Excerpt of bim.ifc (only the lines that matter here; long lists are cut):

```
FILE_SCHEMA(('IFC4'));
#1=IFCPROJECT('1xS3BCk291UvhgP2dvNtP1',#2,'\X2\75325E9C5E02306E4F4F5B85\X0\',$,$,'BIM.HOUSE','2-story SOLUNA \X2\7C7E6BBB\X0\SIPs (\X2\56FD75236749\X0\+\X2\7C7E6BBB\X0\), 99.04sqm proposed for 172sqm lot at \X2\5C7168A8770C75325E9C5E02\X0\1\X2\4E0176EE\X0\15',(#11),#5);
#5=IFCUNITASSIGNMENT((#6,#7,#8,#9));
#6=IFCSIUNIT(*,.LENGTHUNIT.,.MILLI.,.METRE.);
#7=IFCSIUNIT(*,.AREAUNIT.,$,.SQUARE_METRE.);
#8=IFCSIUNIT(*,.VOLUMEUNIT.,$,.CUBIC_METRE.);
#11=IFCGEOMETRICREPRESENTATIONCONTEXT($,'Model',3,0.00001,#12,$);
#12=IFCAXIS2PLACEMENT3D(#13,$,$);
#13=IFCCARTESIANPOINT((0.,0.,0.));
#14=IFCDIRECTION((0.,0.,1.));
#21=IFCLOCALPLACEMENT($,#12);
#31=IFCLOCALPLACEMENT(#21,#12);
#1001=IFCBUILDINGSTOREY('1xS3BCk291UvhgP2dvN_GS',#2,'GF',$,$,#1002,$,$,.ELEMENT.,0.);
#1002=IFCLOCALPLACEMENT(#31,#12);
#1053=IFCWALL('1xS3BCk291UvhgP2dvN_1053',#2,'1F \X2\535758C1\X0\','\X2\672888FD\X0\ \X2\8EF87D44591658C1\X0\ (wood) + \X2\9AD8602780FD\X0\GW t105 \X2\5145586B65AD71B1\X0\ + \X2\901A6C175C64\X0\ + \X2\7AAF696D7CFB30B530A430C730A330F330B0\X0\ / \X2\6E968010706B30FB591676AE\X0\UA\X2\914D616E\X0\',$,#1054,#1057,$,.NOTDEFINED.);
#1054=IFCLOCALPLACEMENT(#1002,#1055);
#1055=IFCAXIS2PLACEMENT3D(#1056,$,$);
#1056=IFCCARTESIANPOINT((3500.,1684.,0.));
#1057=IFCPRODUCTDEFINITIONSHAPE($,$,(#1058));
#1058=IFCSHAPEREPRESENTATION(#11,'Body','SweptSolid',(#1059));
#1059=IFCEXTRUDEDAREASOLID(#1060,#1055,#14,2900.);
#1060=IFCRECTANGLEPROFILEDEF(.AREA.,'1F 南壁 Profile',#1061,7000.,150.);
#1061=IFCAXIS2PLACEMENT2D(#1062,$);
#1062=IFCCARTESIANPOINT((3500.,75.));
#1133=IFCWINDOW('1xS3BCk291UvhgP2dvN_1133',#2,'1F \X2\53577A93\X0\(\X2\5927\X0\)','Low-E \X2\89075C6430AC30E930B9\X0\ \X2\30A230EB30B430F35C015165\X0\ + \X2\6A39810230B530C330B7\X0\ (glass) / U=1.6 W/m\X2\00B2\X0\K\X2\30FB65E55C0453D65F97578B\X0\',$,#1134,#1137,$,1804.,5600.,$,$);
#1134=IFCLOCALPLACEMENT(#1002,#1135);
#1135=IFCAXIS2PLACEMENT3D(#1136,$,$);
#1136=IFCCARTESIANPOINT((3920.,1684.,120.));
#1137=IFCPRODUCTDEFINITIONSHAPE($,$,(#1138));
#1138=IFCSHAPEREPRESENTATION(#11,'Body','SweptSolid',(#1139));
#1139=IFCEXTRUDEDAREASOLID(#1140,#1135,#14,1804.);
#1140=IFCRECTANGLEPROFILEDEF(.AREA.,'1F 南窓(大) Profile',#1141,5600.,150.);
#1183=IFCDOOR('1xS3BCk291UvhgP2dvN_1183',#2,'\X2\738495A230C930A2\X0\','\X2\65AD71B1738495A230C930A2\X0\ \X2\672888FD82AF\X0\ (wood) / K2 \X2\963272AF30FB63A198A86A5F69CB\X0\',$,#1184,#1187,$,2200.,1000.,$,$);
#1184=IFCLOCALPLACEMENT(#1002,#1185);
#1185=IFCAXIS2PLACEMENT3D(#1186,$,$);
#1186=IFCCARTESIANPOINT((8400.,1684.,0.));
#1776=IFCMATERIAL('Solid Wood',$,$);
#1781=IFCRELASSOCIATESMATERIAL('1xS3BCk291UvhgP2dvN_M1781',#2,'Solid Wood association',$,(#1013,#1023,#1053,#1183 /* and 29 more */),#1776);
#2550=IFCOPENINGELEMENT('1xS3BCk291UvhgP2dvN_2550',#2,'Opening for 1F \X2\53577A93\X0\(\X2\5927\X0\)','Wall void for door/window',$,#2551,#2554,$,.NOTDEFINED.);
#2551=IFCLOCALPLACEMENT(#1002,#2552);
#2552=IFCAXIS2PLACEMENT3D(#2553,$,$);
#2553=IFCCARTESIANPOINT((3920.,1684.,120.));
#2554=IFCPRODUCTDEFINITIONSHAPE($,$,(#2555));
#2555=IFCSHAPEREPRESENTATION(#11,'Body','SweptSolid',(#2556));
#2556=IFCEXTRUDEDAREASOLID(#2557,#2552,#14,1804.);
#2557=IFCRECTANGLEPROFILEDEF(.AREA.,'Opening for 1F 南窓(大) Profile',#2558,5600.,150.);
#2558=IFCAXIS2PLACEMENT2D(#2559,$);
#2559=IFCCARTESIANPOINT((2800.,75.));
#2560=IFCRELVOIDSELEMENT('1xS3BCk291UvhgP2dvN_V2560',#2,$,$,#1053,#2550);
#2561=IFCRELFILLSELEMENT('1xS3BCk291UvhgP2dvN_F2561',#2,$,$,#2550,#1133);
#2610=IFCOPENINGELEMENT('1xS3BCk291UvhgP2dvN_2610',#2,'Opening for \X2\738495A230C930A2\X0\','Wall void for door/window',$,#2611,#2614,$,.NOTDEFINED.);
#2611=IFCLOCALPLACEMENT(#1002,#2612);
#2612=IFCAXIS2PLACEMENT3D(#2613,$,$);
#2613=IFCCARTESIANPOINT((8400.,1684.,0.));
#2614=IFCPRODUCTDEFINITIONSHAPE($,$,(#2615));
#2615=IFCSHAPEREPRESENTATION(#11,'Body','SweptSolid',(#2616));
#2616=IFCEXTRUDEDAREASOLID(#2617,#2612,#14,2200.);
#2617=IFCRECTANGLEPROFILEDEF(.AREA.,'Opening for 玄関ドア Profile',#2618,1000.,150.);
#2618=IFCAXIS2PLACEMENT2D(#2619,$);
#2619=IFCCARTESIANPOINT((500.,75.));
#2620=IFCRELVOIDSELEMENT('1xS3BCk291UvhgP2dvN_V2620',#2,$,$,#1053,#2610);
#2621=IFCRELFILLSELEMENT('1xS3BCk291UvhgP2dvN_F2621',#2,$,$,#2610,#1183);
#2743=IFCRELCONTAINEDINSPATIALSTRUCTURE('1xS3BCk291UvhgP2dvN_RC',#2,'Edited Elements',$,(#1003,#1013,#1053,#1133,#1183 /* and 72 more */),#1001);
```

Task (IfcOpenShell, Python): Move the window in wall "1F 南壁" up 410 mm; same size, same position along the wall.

```python
import numpy as np
import ifcopenshell
import ifcopenshell.api.geometry
import ifcopenshell.util.placement
import ifcopenshell.util.unit

model = ifcopenshell.open("bim.ifc")
unit_scale = ifcopenshell.util.unit.calculate_unit_scale(model)

window = model.by_guid("1xS3BCk291UvhgP2dvN_1133")
opening = window.FillsVoids[0].RelatingOpeningElement
dz = 0.41 / unit_scale

shift = np.array([0.0, 0.0, dz])
# The window is not placed relative to its opening, so move both.
for product in (opening, window):
    matrix = ifcopenshell.util.placement.get_local_placement(product.ObjectPlacement)
    matrix[:3, 3] += shift
    ifcopenshell.api.geometry.edit_object_placement(model, product=product, matrix=matrix, is_si=False)

print(f"moved by {dz * unit_scale:+.3f} m")

model.write("bim-out.ifc")
```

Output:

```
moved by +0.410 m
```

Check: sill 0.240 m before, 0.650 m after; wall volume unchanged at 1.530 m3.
